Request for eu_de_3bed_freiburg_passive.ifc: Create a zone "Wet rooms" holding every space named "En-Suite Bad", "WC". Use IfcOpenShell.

First a look at what the model holds.

```python
import ifcopenshell

model = ifcopenshell.open("eu_de_3bed_freiburg_passive.ifc")
print(model.schema)
seen = {}
for space in model.by_type("IfcSpace"):
    seen[space.LongName] = seen.get(space.LongName, 0) + 1
for name, count in sorted(seen.items(), key=str):
    print(count, "x", name)
print("zones:", [z.Name for z in model.by_type("IfcZone")][:20])
```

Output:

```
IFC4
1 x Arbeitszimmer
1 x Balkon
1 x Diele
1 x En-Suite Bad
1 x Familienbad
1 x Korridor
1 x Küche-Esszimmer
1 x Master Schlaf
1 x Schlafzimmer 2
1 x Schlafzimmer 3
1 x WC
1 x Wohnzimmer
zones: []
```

```python
import ifcopenshell
import ifcopenshell.api.group
import ifcopenshell.api.root

model = ifcopenshell.open("eu_de_3bed_freiburg_passive.ifc")

names = {"En-Suite Bad", "WC"}
spaces = [s for s in model.by_type("IfcSpace") if s.LongName in names]

zone = ifcopenshell.api.root.create_entity(model, ifc_class="IfcZone", name="Wet rooms")
ifcopenshell.api.group.assign_group(model, products=spaces, group=zone)
print(len(spaces), "spaces in", zone.Name)

model.write("eu_de_3bed_freiburg_passive_updated.ifc")
```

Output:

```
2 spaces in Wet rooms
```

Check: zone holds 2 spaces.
